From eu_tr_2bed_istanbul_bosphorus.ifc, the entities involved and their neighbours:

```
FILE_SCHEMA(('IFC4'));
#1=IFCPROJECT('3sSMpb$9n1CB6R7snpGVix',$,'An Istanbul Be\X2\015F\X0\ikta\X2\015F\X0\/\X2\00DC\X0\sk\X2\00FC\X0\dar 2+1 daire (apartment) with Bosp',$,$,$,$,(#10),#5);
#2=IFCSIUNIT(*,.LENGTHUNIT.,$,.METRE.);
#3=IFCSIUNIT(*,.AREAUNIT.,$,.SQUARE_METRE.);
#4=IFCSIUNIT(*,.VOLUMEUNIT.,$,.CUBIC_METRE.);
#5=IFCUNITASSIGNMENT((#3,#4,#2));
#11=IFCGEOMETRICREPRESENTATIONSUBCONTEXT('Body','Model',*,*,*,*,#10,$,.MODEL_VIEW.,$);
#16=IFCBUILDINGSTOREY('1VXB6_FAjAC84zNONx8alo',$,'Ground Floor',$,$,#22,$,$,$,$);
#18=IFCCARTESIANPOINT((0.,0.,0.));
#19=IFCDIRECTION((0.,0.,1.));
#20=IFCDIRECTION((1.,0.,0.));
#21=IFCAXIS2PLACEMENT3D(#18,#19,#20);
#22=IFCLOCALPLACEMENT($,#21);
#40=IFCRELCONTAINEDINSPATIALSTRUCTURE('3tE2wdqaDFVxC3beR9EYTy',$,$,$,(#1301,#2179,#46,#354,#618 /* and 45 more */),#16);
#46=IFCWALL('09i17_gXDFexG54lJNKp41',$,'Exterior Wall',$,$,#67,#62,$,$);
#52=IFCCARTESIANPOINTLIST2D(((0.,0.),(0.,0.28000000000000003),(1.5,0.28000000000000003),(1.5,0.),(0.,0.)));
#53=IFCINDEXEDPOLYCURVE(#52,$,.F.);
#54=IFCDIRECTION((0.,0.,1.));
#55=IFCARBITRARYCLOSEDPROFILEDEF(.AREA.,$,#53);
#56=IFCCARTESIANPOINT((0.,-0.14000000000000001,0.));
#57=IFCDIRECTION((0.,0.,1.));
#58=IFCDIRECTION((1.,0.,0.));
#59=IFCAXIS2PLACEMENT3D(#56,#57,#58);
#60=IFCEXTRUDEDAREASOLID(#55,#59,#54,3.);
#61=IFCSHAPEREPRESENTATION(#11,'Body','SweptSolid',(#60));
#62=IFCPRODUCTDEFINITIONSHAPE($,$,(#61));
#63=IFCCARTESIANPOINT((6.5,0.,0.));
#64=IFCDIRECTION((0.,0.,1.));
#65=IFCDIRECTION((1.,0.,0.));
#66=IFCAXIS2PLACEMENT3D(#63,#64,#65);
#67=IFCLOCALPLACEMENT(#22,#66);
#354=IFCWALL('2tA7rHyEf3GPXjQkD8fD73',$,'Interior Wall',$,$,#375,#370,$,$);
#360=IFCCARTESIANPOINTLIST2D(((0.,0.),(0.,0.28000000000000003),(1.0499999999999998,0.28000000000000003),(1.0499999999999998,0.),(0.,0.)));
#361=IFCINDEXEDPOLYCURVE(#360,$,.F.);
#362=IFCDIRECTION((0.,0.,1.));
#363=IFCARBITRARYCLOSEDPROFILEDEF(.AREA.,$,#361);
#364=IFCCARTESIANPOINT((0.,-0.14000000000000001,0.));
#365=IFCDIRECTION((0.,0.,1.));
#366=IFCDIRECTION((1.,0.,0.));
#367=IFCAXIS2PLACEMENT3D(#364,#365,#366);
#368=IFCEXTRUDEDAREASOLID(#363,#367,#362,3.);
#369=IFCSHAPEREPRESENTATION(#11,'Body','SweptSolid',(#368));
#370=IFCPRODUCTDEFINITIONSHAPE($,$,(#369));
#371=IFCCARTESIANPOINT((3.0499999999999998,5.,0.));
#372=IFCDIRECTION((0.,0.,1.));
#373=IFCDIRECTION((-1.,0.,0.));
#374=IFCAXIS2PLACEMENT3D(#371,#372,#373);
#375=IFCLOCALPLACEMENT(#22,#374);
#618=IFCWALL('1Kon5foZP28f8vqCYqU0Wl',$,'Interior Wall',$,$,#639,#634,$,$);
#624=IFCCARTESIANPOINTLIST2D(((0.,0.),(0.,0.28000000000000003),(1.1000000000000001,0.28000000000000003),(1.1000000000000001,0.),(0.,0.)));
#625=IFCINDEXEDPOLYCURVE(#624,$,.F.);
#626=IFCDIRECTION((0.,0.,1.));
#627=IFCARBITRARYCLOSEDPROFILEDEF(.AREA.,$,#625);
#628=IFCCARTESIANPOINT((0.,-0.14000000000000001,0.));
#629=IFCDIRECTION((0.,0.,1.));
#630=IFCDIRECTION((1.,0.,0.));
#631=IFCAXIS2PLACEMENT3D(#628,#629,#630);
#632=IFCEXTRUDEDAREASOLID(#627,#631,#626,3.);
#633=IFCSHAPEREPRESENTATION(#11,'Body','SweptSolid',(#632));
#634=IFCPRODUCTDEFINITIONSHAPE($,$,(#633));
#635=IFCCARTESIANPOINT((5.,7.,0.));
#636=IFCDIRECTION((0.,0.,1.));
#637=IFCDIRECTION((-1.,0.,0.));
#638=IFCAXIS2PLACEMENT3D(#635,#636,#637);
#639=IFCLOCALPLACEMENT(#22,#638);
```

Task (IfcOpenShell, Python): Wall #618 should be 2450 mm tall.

```python
import ifcopenshell
import ifcopenshell.geom
import ifcopenshell.util.representation
import ifcopenshell.util.shape
import ifcopenshell.util.unit

model = ifcopenshell.open("eu_tr_2bed_istanbul_bosphorus.ifc")
unit_scale = ifcopenshell.util.unit.calculate_unit_scale(model)
settings = ifcopenshell.geom.settings()


def volume(element):
    """Net volume in cubic metres, openings subtracted."""
    shape = ifcopenshell.geom.create_shape(settings, element)
    return ifcopenshell.util.shape.get_volume(shape.geometry)


wall = model.by_guid("1Kon5foZP28f8vqCYqU0Wl")
before = volume(wall)

body = ifcopenshell.util.representation.get_representation(wall, "Model", "Body")
solid = body.Items[0]
old_height = solid.Depth
solid.Depth = 2.45 / unit_scale
after = volume(wall)

print(f"height {old_height:g} -> {solid.Depth:g}, volume {before:.3f} -> {after:.3f} m3")

model.write("eu_tr_2bed_istanbul_bosphorus-out.ifc")
```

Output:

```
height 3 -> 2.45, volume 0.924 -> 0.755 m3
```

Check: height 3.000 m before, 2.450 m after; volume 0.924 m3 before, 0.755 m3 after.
